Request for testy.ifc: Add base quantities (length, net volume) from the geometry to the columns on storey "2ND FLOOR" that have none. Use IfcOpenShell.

First a look at what the model holds.

```python
import ifcopenshell
import ifcopenshell.util.element
import ifcopenshell.util.unit

model = ifcopenshell.open("testy.ifc")
print(model.schema)
for unit_type in ("LENGTHUNIT", "AREAUNIT", "VOLUMEUNIT"):
    print(unit_type, ifcopenshell.util.unit.calculate_unit_scale(model, unit_type))
storey = next(s for s in model.by_type("IfcBuildingStorey") if s.Name == "2ND FLOOR")
columns = [e for e in ifcopenshell.util.element.get_decomposition(storey) if e.is_a("IfcColumn")]
for e in sorted(columns, key=lambda e: e.id()):
    print(e.id(), e.is_a(), e.Name, list(ifcopenshell.util.element.get_psets(e, qtos_only=True)), sep=" | ")
```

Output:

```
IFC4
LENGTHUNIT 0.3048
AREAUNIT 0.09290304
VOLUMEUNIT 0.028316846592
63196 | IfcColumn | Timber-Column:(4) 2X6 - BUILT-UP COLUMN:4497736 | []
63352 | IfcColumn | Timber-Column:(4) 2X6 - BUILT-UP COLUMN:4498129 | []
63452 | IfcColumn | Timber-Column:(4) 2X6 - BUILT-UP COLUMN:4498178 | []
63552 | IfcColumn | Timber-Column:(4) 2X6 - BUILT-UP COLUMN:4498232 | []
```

```python
import ifcopenshell
import ifcopenshell.api.pset
import ifcopenshell.geom
import ifcopenshell.util.element
import ifcopenshell.util.shape
import ifcopenshell.util.unit

model = ifcopenshell.open("testy.ifc")
unit_scale = ifcopenshell.util.unit.calculate_unit_scale(model)
volume_scale = ifcopenshell.util.unit.calculate_unit_scale(model, "VOLUMEUNIT")
settings = ifcopenshell.geom.settings()

storey = next(s for s in model.by_type("IfcBuildingStorey") if s.Name == "2ND FLOOR")
columns = [e for e in ifcopenshell.util.element.get_decomposition(storey) if e.is_a("IfcColumn")]

for e in sorted(columns, key=lambda e: e.id()):
    if ifcopenshell.util.element.get_psets(e, qtos_only=True, should_inherit=False):
        continue
    # Geometry comes back in metres, in the element's own axes.
    shape = ifcopenshell.geom.create_shape(settings, e)
    values = {
        "Length": ifcopenshell.util.shape.get_z(shape.geometry) / unit_scale,
        "NetVolume": ifcopenshell.util.shape.get_volume(shape.geometry) / volume_scale,
    }
    qto = ifcopenshell.api.pset.add_qto(model, product=e, name="Qto_ColumnBaseQuantities")
    ifcopenshell.api.pset.edit_qto(model, qto=qto, properties=values)
    print(e.id(), {k: round(v, 3) for k, v in values.items()})

model.write("testy_updated.ifc")
```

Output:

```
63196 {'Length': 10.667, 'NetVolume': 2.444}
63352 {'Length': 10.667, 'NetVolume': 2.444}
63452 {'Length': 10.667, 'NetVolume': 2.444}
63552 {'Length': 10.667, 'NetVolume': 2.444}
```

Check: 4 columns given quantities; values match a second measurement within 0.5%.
